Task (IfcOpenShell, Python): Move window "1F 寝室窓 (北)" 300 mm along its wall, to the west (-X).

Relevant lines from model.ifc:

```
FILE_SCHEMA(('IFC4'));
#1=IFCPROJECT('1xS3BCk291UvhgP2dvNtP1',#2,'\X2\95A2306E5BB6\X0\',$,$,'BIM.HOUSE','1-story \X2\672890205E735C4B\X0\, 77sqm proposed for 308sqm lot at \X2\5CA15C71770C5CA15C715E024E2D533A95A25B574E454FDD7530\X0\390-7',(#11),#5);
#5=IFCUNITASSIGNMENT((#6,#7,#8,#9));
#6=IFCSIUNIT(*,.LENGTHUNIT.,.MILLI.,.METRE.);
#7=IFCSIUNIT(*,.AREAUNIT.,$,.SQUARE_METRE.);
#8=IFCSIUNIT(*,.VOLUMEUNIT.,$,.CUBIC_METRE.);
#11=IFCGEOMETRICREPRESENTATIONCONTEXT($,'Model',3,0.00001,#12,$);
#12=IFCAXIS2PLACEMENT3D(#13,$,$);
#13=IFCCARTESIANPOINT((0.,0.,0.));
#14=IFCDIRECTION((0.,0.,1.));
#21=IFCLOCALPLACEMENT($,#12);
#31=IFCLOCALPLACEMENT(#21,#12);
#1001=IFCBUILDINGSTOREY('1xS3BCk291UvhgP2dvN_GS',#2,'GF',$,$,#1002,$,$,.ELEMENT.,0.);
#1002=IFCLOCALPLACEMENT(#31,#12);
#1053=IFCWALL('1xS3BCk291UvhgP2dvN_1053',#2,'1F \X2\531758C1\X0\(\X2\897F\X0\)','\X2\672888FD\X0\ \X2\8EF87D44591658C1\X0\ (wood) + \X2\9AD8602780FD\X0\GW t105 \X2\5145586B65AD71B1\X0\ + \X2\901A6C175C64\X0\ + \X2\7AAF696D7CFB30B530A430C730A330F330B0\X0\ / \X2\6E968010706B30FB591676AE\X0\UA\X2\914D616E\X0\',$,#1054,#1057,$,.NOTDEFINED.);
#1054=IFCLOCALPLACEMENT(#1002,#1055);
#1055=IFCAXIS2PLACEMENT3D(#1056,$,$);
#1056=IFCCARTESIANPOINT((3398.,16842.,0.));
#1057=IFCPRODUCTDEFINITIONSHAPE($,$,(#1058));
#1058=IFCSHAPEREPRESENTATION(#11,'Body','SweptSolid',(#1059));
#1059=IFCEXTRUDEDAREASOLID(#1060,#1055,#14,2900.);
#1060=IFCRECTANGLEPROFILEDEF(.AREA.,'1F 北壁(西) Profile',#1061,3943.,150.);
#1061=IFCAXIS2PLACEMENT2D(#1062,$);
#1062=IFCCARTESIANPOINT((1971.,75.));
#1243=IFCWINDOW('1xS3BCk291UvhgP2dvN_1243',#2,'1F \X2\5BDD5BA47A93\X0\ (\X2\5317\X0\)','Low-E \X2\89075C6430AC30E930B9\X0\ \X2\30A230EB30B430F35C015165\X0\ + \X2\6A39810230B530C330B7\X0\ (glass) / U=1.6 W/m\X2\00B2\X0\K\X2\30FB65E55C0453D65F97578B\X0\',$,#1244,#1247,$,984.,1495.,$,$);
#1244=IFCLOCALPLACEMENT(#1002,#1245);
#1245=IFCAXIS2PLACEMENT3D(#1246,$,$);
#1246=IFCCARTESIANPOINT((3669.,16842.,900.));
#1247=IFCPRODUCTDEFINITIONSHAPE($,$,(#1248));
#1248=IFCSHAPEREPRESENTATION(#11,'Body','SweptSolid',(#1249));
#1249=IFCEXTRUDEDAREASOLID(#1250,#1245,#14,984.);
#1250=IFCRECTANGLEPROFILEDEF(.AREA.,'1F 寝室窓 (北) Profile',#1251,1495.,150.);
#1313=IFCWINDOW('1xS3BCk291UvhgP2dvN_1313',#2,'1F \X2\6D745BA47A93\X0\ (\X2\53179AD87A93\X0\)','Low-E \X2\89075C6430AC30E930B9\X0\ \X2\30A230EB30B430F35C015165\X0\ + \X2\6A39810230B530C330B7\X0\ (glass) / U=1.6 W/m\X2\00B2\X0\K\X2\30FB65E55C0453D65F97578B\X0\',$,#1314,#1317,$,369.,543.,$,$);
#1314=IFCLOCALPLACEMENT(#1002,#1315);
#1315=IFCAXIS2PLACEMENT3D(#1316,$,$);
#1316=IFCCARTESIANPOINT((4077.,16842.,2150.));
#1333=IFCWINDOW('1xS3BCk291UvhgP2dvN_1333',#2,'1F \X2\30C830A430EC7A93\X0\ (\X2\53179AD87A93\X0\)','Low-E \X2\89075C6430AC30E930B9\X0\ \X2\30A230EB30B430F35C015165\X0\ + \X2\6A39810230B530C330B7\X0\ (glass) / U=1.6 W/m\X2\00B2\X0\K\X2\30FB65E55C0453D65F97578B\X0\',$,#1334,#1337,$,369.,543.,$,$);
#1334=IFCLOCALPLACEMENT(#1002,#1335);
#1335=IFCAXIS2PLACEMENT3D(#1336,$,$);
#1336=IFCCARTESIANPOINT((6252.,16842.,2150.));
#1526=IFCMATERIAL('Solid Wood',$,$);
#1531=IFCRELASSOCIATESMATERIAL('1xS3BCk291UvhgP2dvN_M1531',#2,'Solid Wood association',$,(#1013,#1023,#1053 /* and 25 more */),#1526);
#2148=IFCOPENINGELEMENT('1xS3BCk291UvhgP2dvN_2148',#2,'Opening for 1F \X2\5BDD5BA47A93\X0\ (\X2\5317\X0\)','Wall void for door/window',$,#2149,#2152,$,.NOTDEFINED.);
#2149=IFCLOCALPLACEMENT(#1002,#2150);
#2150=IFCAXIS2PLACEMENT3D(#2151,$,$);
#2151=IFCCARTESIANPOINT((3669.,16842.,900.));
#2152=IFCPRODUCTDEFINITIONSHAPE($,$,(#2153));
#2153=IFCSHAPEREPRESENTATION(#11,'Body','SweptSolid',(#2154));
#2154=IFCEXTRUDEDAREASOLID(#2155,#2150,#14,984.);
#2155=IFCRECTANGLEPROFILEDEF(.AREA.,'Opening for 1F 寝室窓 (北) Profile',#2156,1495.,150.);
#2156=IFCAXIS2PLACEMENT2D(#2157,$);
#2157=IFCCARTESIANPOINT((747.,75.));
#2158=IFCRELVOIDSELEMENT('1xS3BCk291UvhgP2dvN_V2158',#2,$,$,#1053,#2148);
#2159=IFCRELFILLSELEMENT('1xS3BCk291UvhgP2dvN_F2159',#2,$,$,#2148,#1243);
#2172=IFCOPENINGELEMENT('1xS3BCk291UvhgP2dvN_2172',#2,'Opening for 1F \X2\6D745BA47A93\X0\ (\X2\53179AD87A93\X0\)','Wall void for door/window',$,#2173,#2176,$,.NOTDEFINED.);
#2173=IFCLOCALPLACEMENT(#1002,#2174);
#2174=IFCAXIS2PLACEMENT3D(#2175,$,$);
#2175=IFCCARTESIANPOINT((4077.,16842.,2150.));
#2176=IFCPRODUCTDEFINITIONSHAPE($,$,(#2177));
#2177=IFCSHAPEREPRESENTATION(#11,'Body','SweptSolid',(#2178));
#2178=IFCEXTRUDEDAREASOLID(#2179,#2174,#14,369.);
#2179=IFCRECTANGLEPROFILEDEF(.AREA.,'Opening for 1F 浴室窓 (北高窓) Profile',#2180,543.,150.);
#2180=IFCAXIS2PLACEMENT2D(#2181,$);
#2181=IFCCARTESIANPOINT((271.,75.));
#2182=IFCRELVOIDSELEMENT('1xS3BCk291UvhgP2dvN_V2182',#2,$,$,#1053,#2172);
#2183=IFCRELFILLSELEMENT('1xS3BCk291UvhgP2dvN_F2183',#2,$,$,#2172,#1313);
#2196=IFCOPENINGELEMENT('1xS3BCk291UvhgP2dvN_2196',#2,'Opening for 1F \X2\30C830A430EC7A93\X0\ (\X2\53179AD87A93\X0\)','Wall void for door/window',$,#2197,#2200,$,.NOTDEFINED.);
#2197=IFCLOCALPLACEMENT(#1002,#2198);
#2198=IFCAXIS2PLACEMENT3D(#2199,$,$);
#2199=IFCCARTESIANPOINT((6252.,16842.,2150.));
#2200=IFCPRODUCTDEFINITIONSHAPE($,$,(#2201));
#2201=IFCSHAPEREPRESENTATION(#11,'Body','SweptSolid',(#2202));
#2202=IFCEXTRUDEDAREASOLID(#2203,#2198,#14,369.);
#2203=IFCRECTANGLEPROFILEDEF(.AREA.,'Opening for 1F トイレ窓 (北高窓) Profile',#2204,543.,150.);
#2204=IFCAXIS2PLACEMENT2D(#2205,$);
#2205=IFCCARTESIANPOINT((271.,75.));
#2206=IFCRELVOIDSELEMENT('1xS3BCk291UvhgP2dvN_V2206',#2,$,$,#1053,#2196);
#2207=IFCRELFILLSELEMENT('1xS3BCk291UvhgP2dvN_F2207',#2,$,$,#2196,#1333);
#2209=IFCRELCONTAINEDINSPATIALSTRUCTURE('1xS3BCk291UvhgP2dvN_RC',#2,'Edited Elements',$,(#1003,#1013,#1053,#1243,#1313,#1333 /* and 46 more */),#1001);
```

```python
import ifcopenshell
import ifcopenshell.api.geometry
import ifcopenshell.util.placement
import ifcopenshell.util.unit

model = ifcopenshell.open("model.ifc")
unit_scale = ifcopenshell.util.unit.calculate_unit_scale(model)

window = model.by_guid("1xS3BCk291UvhgP2dvN_1243")
opening = window.FillsVoids[0].RelatingOpeningElement
wall = opening.VoidsElements[0].RelatingBuildingElement

wall_matrix = ifcopenshell.util.placement.get_local_placement(wall.ObjectPlacement)
shift = wall_matrix[:3, 0] * -0.3 / unit_scale
before = ifcopenshell.util.placement.get_local_placement(window.ObjectPlacement)[:3, 3].copy()

# The window is not placed relative to its opening, so move both.
for product in (opening, window):
    matrix = ifcopenshell.util.placement.get_local_placement(product.ObjectPlacement)
    matrix[:3, 3] += shift
    ifcopenshell.api.geometry.edit_object_placement(model, product=product, matrix=matrix, is_si=False)

after = ifcopenshell.util.placement.get_local_placement(window.ObjectPlacement)[:3, 3]
print("window moved by", (after - before).round(3) + 0.0)

model.write("model_v2.ifc")
```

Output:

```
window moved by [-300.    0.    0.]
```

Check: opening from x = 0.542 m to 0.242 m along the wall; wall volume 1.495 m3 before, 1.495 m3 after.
